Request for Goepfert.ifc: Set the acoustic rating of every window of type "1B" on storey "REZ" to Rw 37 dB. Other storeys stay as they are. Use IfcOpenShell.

First a look at what the model holds.

```python
import ifcopenshell
import ifcopenshell.util.element

model = ifcopenshell.open("Goepfert.ifc")
print(model.schema)
storey = next(s for s in model.by_type("IfcBuildingStorey") if s.Name == "REZ")
windows = [e for e in ifcopenshell.util.element.get_decomposition(storey) if e.is_a("IfcWindow")]
seen = {}
for e in windows:
    element_type = ifcopenshell.util.element.get_type(e)
    key = (element_type.Name if element_type != e and element_type else None, ifcopenshell.util.element.get_pset(e, "Pset_WindowCommon", "AcousticRating"))
    seen[key] = seen.get(key, 0) + 1
for (name, value), count in sorted(seen.items(), key=str):
    print(count, "x", name, "|", value)
```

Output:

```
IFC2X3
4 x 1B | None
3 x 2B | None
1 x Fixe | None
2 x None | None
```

```python
import ifcopenshell
import ifcopenshell.api.pset
import ifcopenshell.util.element

model = ifcopenshell.open("Goepfert.ifc")

storey = next(s for s in model.by_type("IfcBuildingStorey") if s.Name == "REZ")
windows = [e for e in ifcopenshell.util.element.get_decomposition(storey) if e.is_a("IfcWindow")]

count = 0
for e in windows:
    element_type = ifcopenshell.util.element.get_type(e)
    if element_type in (None, e) or element_type.Name != "1B":
        continue
    # add_pset returns the element's existing set when there is one.
    pset = ifcopenshell.api.pset.add_pset(model, product=e, name="Pset_WindowCommon")
    ifcopenshell.api.pset.edit_pset(model, pset=pset, properties={"AcousticRating": "Rw 37 dB"})
    count += 1

print(count, "windows updated")

model.write("Goepfert_updated.ifc")
```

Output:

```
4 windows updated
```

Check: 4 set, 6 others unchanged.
